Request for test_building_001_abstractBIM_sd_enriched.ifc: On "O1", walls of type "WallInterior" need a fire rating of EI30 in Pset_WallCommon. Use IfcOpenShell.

First a look at what the model holds.

```python
import ifcopenshell
import ifcopenshell.util.element

model = ifcopenshell.open("test_building_001_abstractBIM_sd_enriched.ifc")
print(model.schema)
storey = next(s for s in model.by_type("IfcBuildingStorey") if s.Name == "O1")
walls = [e for e in ifcopenshell.util.element.get_decomposition(storey) if e.is_a("IfcWall")]
seen = {}
for e in walls:
    element_type = ifcopenshell.util.element.get_type(e)
    key = (element_type.Name if element_type != e and element_type else None, ifcopenshell.util.element.get_pset(e, "Pset_WallCommon", "FireRating"))
    seen[key] = seen.get(key, 0) + 1
for (name, value), count in sorted(seen.items(), key=str):
    print(count, "x", name, "|", value)
```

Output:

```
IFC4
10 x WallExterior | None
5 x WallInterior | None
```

```python
import ifcopenshell
import ifcopenshell.api.pset
import ifcopenshell.util.element

model = ifcopenshell.open("test_building_001_abstractBIM_sd_enriched.ifc")

storey = next(s for s in model.by_type("IfcBuildingStorey") if s.Name == "O1")
walls = [e for e in ifcopenshell.util.element.get_decomposition(storey) if e.is_a("IfcWall")]

count = 0
for e in walls:
    element_type = ifcopenshell.util.element.get_type(e)
    if element_type in (None, e) or element_type.Name != "WallInterior":
        continue
    # add_pset returns the element's existing set when there is one.
    pset = ifcopenshell.api.pset.add_pset(model, product=e, name="Pset_WallCommon")
    ifcopenshell.api.pset.edit_pset(model, pset=pset, properties={"FireRating": "EI30"})
    count += 1

print(count, "walls updated")

model.write("test_building_001_abstractBIM_sd_enriched_edited.ifc")
```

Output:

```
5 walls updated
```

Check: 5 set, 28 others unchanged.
